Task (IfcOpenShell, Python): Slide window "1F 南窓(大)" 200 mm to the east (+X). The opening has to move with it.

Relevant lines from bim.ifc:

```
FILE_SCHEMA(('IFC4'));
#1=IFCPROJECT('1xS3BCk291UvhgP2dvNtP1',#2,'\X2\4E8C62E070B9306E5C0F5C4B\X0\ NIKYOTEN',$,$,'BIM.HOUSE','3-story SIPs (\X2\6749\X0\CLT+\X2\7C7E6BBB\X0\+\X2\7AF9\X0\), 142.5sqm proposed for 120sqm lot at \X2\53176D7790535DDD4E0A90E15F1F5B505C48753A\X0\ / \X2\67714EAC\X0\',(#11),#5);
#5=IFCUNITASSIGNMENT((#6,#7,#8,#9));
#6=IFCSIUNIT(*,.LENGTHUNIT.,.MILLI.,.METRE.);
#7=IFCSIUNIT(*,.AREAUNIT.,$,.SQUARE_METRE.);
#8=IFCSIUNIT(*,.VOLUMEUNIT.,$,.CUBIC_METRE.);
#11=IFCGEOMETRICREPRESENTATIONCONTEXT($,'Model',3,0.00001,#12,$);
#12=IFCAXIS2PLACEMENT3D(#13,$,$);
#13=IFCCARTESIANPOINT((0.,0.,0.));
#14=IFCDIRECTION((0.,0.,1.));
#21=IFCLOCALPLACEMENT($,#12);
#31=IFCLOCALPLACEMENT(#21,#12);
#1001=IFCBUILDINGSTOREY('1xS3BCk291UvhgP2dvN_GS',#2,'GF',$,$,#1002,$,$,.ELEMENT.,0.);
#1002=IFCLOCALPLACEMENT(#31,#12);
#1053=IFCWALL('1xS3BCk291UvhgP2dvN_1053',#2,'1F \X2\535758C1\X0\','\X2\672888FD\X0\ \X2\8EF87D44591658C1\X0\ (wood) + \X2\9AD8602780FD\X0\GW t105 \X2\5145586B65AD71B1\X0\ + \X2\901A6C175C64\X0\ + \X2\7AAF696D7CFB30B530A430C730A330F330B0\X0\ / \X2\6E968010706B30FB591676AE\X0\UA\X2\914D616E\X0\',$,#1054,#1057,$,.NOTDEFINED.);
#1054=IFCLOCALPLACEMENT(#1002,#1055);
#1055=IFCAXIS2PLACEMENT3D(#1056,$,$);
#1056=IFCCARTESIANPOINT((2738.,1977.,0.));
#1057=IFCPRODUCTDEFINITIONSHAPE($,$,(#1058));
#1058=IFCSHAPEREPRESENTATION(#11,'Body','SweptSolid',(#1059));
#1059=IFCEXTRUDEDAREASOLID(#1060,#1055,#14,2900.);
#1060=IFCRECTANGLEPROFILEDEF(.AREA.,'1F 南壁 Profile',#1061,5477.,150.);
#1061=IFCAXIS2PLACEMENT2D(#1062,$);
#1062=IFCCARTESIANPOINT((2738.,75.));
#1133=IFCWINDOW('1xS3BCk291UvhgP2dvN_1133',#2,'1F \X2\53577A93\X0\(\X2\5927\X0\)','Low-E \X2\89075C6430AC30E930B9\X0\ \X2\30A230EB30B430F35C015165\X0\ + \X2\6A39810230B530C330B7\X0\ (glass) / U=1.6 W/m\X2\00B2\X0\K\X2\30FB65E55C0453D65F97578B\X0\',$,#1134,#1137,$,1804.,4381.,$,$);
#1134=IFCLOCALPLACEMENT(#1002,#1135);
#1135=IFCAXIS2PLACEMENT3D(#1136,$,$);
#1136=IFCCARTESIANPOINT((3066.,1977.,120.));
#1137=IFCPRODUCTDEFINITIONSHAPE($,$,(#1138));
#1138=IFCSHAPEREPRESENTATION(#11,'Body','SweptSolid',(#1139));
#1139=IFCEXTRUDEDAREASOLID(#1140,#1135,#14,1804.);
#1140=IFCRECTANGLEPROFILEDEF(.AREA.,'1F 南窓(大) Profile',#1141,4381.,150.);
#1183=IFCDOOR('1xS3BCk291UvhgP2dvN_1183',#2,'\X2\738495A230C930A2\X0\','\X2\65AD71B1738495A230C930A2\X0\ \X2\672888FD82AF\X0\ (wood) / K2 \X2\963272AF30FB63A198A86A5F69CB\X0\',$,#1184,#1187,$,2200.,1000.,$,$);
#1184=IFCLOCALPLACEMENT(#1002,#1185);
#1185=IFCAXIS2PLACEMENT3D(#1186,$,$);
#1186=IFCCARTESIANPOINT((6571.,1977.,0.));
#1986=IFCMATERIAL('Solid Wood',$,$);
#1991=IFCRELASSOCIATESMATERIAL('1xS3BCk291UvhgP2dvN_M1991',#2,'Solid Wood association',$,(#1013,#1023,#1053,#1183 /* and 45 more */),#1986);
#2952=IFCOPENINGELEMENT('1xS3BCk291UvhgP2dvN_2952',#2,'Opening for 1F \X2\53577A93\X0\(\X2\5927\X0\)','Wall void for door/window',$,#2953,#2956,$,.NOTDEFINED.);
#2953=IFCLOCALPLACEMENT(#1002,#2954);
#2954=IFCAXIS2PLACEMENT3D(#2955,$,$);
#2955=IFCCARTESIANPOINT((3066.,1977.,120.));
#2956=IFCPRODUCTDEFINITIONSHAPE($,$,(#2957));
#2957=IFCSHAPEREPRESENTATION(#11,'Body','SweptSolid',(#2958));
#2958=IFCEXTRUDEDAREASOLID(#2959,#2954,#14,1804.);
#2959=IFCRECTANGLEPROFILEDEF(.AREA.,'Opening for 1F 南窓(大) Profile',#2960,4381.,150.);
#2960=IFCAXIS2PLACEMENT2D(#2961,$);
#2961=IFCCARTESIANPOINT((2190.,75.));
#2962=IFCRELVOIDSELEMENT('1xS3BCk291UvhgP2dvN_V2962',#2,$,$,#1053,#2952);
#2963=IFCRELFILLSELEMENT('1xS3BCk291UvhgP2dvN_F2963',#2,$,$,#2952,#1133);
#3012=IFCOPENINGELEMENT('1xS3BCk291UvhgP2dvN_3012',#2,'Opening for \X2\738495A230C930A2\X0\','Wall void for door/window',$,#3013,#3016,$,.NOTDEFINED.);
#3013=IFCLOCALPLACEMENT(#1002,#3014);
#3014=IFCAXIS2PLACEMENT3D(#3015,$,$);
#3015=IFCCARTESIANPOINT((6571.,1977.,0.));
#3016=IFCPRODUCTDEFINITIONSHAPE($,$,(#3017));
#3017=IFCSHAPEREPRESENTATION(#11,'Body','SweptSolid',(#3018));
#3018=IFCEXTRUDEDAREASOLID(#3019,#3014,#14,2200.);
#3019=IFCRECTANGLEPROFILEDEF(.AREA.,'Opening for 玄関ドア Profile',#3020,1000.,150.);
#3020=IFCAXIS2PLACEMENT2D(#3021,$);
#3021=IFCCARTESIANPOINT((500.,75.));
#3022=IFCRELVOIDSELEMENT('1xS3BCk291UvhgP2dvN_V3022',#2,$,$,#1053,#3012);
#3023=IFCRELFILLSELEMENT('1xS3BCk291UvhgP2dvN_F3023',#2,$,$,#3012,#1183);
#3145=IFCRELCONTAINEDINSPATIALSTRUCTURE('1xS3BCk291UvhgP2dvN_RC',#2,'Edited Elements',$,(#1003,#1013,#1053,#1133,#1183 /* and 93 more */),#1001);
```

```python
import ifcopenshell
import ifcopenshell.api.geometry
import ifcopenshell.util.placement
import ifcopenshell.util.unit

model = ifcopenshell.open("bim.ifc")
unit_scale = ifcopenshell.util.unit.calculate_unit_scale(model)

window = model.by_id(1133)
opening = window.FillsVoids[0].RelatingOpeningElement
wall = opening.VoidsElements[0].RelatingBuildingElement

wall_matrix = ifcopenshell.util.placement.get_local_placement(wall.ObjectPlacement)
shift = wall_matrix[:3, 0] * 0.2 / unit_scale
before = ifcopenshell.util.placement.get_local_placement(window.ObjectPlacement)[:3, 3].copy()

# The window is not placed relative to its opening, so move both.
for product in (opening, window):
    matrix = ifcopenshell.util.placement.get_local_placement(product.ObjectPlacement)
    matrix[:3, 3] += shift
    ifcopenshell.api.geometry.edit_object_placement(model, product=product, matrix=matrix, is_si=False)

after = ifcopenshell.util.placement.get_local_placement(window.ObjectPlacement)[:3, 3]
print("window moved by", (after - before).round(3) + 0.0)

model.write("bim_v2.ifc")
```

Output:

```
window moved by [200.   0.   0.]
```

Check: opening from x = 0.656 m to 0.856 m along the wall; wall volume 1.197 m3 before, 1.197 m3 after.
